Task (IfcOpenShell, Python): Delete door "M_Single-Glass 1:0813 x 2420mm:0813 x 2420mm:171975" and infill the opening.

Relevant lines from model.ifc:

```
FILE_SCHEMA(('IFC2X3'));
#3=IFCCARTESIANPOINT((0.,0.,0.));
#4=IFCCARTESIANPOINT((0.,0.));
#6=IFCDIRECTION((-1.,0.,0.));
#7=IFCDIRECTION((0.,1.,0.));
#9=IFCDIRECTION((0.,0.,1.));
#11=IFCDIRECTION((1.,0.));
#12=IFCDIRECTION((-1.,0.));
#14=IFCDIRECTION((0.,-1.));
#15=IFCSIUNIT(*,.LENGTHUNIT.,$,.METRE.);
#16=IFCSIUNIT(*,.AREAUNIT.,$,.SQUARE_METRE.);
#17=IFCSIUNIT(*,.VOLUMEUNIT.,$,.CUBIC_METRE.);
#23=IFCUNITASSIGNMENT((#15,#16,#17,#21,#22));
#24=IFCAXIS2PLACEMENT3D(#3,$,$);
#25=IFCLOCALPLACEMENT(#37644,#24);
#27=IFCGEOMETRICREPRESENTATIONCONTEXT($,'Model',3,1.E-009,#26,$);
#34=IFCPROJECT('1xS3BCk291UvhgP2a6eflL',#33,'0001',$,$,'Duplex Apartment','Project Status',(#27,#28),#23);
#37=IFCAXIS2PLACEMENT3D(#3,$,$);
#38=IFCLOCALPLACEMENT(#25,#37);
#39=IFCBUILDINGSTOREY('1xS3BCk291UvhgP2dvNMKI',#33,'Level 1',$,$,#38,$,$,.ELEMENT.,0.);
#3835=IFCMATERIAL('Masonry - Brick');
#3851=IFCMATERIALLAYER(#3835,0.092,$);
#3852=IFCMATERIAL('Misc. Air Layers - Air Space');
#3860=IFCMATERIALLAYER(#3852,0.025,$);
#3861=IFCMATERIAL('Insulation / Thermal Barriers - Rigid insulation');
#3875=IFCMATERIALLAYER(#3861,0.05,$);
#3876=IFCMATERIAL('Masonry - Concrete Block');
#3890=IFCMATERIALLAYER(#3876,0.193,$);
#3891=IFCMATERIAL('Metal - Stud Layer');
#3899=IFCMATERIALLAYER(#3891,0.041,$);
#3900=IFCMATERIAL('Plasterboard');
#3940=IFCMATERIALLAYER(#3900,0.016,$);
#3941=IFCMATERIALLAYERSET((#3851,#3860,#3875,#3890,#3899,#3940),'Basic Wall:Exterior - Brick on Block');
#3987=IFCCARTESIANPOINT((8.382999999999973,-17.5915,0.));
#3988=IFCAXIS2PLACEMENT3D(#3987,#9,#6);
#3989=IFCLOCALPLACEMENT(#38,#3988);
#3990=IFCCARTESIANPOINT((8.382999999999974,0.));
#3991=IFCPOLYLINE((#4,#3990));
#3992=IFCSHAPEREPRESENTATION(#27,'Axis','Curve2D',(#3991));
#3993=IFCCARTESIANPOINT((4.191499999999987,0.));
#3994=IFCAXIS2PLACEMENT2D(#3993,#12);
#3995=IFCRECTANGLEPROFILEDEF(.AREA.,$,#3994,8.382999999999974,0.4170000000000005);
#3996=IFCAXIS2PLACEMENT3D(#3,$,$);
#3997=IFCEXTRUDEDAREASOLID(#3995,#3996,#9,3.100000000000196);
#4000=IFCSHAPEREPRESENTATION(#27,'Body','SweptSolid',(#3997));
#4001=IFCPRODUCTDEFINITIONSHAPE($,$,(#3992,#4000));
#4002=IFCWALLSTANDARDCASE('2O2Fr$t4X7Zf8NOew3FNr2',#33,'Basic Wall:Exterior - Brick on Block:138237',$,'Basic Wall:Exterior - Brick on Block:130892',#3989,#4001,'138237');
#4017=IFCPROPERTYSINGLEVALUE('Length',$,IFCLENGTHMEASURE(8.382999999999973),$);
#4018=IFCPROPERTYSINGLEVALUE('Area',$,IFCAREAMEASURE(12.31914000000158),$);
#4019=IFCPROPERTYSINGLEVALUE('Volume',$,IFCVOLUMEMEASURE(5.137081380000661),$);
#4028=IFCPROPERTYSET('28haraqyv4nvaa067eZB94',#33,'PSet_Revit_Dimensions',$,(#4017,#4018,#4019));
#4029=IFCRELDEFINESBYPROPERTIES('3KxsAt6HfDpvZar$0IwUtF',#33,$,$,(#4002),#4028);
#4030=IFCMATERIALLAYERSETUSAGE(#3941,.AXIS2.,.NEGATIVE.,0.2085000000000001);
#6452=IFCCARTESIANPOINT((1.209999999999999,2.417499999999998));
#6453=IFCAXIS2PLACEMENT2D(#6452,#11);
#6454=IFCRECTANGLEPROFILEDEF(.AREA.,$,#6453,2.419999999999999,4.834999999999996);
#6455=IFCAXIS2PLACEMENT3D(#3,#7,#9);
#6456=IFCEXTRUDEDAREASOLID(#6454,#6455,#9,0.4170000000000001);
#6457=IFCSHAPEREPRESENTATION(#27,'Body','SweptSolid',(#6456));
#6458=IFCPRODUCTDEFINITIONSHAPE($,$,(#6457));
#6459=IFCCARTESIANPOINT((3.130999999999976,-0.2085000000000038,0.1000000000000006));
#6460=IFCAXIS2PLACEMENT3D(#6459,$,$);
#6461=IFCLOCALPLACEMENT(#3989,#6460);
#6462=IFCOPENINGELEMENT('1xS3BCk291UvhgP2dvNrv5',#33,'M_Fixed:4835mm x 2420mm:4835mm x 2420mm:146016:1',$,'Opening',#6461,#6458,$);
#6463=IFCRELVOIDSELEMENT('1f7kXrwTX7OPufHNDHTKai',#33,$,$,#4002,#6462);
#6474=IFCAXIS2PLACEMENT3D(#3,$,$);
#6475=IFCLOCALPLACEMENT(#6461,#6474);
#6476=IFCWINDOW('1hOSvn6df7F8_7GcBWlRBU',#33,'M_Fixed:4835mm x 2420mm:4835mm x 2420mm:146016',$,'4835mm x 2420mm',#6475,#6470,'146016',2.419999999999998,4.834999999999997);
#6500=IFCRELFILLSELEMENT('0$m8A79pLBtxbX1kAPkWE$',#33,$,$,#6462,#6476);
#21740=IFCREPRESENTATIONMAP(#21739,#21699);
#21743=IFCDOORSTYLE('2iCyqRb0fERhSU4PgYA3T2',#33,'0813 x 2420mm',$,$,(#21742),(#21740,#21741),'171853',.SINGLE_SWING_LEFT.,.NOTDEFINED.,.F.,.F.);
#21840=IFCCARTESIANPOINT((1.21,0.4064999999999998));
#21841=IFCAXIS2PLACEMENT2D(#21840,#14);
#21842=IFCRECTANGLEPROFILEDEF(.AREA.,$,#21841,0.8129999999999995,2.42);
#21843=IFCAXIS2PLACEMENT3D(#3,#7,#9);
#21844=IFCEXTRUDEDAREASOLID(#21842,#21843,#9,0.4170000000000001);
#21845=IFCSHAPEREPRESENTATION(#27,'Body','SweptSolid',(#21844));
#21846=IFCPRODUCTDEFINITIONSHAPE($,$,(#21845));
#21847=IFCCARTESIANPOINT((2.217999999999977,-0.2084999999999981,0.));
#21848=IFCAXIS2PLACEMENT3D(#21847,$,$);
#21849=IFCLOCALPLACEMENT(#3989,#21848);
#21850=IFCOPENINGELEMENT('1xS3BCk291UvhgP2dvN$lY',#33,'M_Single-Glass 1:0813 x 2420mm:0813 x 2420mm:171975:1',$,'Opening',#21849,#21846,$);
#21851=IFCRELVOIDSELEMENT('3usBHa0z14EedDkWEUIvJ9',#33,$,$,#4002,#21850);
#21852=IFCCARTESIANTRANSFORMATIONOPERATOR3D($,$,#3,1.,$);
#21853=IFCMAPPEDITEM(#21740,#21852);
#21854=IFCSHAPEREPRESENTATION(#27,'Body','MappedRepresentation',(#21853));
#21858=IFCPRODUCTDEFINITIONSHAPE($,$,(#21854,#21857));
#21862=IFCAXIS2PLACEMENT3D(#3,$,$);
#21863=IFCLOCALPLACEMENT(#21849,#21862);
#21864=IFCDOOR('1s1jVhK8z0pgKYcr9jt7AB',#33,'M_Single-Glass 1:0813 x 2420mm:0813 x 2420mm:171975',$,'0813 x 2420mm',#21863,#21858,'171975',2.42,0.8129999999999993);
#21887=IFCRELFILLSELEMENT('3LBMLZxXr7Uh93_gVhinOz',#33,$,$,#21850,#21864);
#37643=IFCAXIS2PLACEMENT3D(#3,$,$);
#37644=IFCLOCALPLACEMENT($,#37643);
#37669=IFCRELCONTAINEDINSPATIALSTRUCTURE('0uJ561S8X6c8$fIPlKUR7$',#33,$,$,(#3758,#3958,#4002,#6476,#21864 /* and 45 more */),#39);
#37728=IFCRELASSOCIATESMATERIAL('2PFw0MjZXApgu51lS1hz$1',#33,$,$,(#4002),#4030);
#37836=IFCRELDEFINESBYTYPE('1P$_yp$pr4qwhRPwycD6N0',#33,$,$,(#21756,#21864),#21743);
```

```python
import ifcopenshell
import ifcopenshell.api.feature
import ifcopenshell.api.pset
import ifcopenshell.api.root
import ifcopenshell.geom
import ifcopenshell.util.element
import ifcopenshell.util.shape
import ifcopenshell.util.unit

model = ifcopenshell.open("model.ifc")
area_scale = ifcopenshell.util.unit.calculate_unit_scale(model, "AREAUNIT")
volume_scale = ifcopenshell.util.unit.calculate_unit_scale(model, "VOLUMEUNIT")
settings = ifcopenshell.geom.settings()


def volume(element):
    """Net volume in cubic metres, openings subtracted."""
    shape = ifcopenshell.geom.create_shape(settings, element)
    return ifcopenshell.util.shape.get_volume(shape.geometry)


door = model.by_guid("1s1jVhK8z0pgKYcr9jt7AB")
opening = door.FillsVoids[0].RelatingOpeningElement
wall = opening.VoidsElements[0].RelatingBuildingElement
before = volume(wall)

ifcopenshell.api.root.remove_product(model, product=door)
ifcopenshell.api.feature.remove_feature(model, feature=opening)

after = volume(wall)
thickness = 0.417  # wall thickness in metres

# Update the wall's stored quantities.
pset = model.by_id(ifcopenshell.util.element.get_pset(wall, "PSet_Revit_Dimensions", should_inherit=False)["id"])
ifcopenshell.api.pset.edit_pset(model, pset=pset, properties={
    "Area": model.create_entity("IfcAreaMeasure", after / thickness / area_scale),
    "Volume": model.create_entity("IfcVolumeMeasure", after / volume_scale),
})

print(f"wall volume {before:.3f} -> {after:.3f} m3")

model.write("model_edited.ifc")
```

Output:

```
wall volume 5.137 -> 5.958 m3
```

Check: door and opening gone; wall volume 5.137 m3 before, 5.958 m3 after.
